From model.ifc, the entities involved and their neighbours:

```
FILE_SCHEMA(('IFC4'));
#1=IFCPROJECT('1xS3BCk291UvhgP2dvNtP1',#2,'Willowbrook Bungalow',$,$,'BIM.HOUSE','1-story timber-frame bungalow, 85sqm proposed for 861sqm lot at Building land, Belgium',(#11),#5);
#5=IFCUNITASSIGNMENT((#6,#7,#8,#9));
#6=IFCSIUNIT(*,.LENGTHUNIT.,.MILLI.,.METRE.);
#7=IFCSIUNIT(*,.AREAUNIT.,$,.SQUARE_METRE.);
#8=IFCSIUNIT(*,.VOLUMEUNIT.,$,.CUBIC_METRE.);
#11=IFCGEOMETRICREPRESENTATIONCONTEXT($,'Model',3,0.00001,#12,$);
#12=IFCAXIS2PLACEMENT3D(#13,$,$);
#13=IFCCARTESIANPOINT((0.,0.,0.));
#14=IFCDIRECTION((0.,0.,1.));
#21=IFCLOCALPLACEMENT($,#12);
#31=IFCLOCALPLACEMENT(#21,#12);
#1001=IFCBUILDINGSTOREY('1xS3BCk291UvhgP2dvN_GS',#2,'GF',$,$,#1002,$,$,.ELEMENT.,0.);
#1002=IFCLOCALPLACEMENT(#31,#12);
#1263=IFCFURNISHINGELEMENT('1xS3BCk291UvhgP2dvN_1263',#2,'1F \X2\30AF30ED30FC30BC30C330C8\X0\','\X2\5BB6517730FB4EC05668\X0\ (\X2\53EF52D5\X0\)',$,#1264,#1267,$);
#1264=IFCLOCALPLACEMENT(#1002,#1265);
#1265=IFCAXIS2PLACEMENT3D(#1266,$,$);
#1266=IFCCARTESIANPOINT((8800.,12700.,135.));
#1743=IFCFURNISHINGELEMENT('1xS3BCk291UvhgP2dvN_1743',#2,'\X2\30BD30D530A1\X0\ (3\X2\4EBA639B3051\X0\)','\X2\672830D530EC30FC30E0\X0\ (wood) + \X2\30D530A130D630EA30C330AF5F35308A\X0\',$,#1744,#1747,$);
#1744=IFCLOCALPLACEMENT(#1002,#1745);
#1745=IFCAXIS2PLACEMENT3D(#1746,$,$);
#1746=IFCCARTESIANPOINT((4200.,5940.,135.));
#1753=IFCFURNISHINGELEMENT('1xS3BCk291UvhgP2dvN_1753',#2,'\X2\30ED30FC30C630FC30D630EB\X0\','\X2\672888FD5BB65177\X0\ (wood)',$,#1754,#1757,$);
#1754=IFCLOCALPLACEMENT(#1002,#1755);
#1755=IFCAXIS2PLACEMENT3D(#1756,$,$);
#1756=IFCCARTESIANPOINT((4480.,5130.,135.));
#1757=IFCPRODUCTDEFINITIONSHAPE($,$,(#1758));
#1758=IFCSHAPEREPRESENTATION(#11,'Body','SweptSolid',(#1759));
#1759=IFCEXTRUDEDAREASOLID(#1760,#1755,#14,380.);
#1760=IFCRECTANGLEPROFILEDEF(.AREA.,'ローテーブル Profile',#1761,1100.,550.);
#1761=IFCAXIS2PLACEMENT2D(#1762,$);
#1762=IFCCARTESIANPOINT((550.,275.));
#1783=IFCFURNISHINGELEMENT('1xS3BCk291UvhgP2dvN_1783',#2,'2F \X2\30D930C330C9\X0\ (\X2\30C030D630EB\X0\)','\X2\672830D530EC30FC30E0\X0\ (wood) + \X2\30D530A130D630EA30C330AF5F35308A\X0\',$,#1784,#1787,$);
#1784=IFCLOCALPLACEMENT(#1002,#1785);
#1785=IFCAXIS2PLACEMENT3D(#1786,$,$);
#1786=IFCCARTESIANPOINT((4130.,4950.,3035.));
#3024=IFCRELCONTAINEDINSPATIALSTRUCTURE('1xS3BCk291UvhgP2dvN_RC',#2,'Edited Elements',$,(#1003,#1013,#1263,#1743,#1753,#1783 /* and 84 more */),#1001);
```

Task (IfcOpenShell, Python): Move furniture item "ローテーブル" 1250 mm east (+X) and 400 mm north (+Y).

```python
import ifcopenshell
import ifcopenshell.api.geometry
import ifcopenshell.util.placement
import ifcopenshell.util.unit

model = ifcopenshell.open("model.ifc")
unit_scale = ifcopenshell.util.unit.calculate_unit_scale(model)

item = model.by_guid("1xS3BCk291UvhgP2dvN_1753")
matrix = ifcopenshell.util.placement.get_local_placement(item.ObjectPlacement)
matrix[0, 3] += 1.25 / unit_scale
matrix[1, 3] += 0.4 / unit_scale
ifcopenshell.api.geometry.edit_object_placement(model, product=item, matrix=matrix, is_si=False)

print(ifcopenshell.util.placement.get_local_placement(item.ObjectPlacement).round(3) + 0.0)

model.write("model_v2.ifc")
```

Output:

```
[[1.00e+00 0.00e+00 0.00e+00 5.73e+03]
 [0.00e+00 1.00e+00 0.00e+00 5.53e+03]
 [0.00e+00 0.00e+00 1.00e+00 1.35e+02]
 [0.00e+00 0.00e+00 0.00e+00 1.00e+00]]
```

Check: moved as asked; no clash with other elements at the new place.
